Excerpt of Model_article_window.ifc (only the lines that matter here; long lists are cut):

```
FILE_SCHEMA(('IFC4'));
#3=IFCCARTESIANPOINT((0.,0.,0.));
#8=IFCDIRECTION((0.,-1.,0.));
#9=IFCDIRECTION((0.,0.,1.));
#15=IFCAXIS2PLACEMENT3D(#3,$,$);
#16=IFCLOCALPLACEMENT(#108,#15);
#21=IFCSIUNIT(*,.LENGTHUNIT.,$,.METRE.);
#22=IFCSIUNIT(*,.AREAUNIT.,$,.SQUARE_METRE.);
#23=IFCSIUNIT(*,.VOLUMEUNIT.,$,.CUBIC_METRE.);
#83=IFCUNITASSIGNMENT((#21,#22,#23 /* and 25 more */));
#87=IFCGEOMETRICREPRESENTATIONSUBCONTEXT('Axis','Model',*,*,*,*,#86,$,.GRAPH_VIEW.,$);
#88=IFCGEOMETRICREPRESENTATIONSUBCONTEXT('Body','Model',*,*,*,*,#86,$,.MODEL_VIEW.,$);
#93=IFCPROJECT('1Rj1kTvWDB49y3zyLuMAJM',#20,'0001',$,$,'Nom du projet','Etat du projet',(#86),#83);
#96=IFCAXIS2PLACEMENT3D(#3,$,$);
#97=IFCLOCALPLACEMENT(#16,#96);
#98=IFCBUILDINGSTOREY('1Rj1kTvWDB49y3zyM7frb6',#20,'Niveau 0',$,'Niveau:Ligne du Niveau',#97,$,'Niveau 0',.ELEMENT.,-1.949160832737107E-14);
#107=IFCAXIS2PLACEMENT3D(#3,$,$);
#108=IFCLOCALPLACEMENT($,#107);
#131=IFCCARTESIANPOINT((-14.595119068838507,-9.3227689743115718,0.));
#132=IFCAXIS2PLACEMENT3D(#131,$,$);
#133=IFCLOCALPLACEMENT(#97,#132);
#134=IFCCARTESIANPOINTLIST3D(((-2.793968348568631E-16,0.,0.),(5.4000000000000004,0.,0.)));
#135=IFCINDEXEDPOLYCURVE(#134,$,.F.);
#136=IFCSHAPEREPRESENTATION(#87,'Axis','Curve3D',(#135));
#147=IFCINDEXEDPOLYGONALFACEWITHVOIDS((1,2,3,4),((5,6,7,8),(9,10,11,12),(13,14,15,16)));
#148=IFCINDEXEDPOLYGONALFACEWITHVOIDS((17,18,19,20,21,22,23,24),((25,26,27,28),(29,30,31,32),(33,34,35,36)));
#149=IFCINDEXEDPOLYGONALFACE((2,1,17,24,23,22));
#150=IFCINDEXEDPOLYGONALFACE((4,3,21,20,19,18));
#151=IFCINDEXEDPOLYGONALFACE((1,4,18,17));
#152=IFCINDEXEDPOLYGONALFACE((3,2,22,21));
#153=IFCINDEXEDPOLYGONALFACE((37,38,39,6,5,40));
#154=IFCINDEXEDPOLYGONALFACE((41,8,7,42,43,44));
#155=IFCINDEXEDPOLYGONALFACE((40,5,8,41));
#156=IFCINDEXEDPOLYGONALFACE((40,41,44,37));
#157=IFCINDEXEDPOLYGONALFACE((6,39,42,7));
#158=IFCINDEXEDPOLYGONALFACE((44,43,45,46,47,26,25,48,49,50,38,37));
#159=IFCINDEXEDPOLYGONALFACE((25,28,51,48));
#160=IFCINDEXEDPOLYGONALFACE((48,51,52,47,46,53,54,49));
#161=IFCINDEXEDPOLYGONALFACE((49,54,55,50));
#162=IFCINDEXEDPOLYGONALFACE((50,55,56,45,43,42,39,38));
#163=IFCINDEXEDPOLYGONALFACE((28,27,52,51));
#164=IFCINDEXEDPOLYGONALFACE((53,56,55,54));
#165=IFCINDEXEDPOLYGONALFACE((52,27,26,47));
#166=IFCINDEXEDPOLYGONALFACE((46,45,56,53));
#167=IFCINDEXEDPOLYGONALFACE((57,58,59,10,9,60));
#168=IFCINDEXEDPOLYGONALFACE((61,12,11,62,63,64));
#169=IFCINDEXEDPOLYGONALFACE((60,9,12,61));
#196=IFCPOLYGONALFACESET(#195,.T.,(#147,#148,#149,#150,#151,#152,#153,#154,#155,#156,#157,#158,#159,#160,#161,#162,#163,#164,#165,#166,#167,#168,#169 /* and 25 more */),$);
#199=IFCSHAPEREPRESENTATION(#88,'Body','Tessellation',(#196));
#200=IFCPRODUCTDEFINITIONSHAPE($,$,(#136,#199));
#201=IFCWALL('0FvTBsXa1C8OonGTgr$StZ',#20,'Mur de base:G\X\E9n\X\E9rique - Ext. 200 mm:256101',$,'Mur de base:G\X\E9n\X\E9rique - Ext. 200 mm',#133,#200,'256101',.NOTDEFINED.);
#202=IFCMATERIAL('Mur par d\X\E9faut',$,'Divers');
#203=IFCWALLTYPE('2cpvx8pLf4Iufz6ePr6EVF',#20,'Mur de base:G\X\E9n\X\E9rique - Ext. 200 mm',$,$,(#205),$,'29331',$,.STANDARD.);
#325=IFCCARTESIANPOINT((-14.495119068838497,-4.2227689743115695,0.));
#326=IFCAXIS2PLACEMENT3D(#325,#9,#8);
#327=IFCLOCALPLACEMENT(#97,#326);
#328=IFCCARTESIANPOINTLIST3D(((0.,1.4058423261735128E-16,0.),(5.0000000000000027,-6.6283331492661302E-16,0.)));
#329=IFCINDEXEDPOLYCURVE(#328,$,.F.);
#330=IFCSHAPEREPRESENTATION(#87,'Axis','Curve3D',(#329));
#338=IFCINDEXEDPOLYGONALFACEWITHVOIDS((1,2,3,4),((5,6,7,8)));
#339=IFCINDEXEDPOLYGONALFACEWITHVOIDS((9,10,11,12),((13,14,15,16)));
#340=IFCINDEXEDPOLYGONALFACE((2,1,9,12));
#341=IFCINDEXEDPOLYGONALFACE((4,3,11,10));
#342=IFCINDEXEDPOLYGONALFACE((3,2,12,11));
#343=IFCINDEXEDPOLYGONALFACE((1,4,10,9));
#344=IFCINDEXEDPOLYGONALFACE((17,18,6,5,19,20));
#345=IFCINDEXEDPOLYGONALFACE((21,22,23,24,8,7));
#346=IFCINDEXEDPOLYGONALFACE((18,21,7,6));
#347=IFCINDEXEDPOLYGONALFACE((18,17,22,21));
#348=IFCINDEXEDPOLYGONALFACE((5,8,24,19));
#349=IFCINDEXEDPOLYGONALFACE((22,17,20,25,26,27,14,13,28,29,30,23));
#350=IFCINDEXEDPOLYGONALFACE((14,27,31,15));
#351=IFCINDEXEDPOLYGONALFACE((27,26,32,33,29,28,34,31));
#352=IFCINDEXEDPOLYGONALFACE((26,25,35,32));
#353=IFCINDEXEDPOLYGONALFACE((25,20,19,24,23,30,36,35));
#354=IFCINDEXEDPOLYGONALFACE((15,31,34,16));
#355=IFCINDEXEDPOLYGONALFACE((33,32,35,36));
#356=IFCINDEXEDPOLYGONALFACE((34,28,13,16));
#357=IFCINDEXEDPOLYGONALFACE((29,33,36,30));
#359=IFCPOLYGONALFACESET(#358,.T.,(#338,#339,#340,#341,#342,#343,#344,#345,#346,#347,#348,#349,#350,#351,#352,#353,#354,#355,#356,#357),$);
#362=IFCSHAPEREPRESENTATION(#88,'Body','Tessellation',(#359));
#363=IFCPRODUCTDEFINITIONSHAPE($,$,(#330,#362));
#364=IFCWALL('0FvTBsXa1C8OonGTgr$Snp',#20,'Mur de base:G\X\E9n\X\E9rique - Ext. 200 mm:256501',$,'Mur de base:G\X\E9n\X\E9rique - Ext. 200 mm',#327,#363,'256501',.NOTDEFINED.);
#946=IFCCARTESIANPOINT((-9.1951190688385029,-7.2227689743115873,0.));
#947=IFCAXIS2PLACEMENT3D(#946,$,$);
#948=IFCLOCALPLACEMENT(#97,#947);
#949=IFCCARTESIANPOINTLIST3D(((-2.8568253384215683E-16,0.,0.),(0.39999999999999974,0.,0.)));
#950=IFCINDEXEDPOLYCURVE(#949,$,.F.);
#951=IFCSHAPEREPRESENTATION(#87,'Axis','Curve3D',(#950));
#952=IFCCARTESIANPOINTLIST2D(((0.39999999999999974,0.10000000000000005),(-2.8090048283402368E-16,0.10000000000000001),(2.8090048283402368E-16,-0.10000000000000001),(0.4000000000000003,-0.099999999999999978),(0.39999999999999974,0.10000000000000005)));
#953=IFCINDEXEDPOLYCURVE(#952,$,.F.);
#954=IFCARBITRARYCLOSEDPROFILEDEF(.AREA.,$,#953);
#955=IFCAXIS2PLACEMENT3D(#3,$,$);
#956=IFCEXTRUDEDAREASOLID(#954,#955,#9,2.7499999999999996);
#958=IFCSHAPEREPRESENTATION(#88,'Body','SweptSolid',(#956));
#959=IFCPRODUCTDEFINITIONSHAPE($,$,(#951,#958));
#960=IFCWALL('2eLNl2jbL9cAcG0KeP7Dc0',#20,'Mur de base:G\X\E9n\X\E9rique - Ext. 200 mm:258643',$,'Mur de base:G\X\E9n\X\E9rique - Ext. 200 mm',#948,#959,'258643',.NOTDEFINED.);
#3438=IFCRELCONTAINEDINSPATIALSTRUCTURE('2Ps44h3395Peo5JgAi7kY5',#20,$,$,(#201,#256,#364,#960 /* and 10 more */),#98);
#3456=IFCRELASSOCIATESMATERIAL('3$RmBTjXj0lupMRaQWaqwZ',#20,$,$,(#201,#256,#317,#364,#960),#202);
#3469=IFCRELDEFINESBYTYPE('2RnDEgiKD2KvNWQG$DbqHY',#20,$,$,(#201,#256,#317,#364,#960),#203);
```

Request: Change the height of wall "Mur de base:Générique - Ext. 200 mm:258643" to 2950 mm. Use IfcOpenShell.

```python
import ifcopenshell
import ifcopenshell.geom
import ifcopenshell.util.representation
import ifcopenshell.util.shape
import ifcopenshell.util.unit

model = ifcopenshell.open("Model_article_window.ifc")
unit_scale = ifcopenshell.util.unit.calculate_unit_scale(model)
settings = ifcopenshell.geom.settings()


def volume(element):
    """Net volume in cubic metres, openings subtracted."""
    shape = ifcopenshell.geom.create_shape(settings, element)
    return ifcopenshell.util.shape.get_volume(shape.geometry)


wall = model.by_id(960)
before = volume(wall)

body = ifcopenshell.util.representation.get_representation(wall, "Model", "Body")
solid = body.Items[0]
old_height = solid.Depth
solid.Depth = 2.95 / unit_scale
after = volume(wall)

print(f"height {old_height:g} -> {solid.Depth:g}, volume {before:.3f} -> {after:.3f} m3")

model.write("Model_article_window_v2.ifc")
```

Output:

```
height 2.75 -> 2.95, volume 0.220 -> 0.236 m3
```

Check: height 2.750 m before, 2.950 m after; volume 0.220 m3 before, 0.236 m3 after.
